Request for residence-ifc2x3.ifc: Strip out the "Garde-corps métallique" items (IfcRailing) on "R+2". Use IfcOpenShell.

First a look at what the model holds.

```python
import ifcopenshell
import ifcopenshell.util.element

model = ifcopenshell.open("residence-ifc2x3.ifc")
print(model.schema)
storey = next(s for s in model.by_type("IfcBuildingStorey") if s.Name == "R+2")
railings = [e for e in ifcopenshell.util.element.get_decomposition(storey) if e.is_a("IfcRailing")]
seen = {}
for e in railings:
    element_type = ifcopenshell.util.element.get_type(e)
    name = element_type.Name if element_type not in (None, e) else None
    seen[name] = seen.get(name, 0) + 1
for name, count in sorted(seen.items(), key=str):
    print(count, "x", name)
```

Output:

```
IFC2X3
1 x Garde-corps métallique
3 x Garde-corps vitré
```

```python
import ifcopenshell
import ifcopenshell.api.root
import ifcopenshell.util.element

model = ifcopenshell.open("residence-ifc2x3.ifc")

storey = next(s for s in model.by_type("IfcBuildingStorey") if s.Name == "R+2")
railings = [e for e in ifcopenshell.util.element.get_decomposition(storey) if e.is_a("IfcRailing")]
targets = [e for e in railings if (t := ifcopenshell.util.element.get_type(e)) not in (None, e) and t.Name == "Garde-corps métallique"]

for e in targets:
    ifcopenshell.api.root.remove_product(model, product=e)
print(len(targets), "removed")

model.write("residence-ifc2x3_updated.ifc")
```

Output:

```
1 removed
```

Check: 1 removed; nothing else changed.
